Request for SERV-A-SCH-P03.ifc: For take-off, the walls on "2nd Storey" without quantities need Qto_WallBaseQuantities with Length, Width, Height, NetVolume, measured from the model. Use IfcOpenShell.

First a look at what the model holds.

```python
import ifcopenshell
import ifcopenshell.util.element
import ifcopenshell.util.unit

model = ifcopenshell.open("SERV-A-SCH-P03.ifc")
print(model.schema)
for unit_type in ("LENGTHUNIT", "AREAUNIT", "VOLUMEUNIT"):
    print(unit_type, ifcopenshell.util.unit.calculate_unit_scale(model, unit_type))
storey = next(s for s in model.by_type("IfcBuildingStorey") if s.Name == "2nd Storey")
walls = [e for e in ifcopenshell.util.element.get_decomposition(storey) if e.is_a("IfcWall")]
for e in sorted(walls, key=lambda e: e.id()):
    print(e.id(), e.is_a(), e.Name, list(ifcopenshell.util.element.get_psets(e, qtos_only=True)), sep=" | ")
```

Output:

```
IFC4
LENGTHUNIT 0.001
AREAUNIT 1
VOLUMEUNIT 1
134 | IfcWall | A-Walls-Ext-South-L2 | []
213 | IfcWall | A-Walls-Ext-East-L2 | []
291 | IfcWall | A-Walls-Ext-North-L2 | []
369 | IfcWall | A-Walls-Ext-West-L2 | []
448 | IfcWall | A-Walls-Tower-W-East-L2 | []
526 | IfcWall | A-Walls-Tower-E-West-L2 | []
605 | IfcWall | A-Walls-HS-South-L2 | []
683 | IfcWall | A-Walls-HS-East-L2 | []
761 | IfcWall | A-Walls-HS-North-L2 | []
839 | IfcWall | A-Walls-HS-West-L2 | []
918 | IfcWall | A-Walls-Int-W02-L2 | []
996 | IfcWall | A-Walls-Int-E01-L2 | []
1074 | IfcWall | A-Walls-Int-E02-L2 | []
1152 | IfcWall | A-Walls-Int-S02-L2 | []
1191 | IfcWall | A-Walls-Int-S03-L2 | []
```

```python
import ifcopenshell
import ifcopenshell.api.pset
import ifcopenshell.geom
import ifcopenshell.util.element
import ifcopenshell.util.shape
import ifcopenshell.util.unit

model = ifcopenshell.open("SERV-A-SCH-P03.ifc")
unit_scale = ifcopenshell.util.unit.calculate_unit_scale(model)
volume_scale = ifcopenshell.util.unit.calculate_unit_scale(model, "VOLUMEUNIT")
settings = ifcopenshell.geom.settings()

storey = next(s for s in model.by_type("IfcBuildingStorey") if s.Name == "2nd Storey")
walls = [e for e in ifcopenshell.util.element.get_decomposition(storey) if e.is_a("IfcWall")]

for e in sorted(walls, key=lambda e: e.id()):
    if ifcopenshell.util.element.get_psets(e, qtos_only=True, should_inherit=False):
        continue
    # Geometry comes back in metres, in the element's own axes.
    shape = ifcopenshell.geom.create_shape(settings, e)
    values = {
        "Length": ifcopenshell.util.shape.get_x(shape.geometry) / unit_scale,
        "Width": ifcopenshell.util.shape.get_y(shape.geometry) / unit_scale,
        "Height": ifcopenshell.util.shape.get_z(shape.geometry) / unit_scale,
        "NetVolume": ifcopenshell.util.shape.get_volume(shape.geometry) / volume_scale,
    }
    qto = ifcopenshell.api.pset.add_qto(model, product=e, name="Qto_WallBaseQuantities")
    ifcopenshell.api.pset.edit_qto(model, qto=qto, properties=values)
    print(e.id(), {k: round(v, 3) for k, v in values.items()})

model.write("SERV-A-SCH-P03_edited.ifc")
```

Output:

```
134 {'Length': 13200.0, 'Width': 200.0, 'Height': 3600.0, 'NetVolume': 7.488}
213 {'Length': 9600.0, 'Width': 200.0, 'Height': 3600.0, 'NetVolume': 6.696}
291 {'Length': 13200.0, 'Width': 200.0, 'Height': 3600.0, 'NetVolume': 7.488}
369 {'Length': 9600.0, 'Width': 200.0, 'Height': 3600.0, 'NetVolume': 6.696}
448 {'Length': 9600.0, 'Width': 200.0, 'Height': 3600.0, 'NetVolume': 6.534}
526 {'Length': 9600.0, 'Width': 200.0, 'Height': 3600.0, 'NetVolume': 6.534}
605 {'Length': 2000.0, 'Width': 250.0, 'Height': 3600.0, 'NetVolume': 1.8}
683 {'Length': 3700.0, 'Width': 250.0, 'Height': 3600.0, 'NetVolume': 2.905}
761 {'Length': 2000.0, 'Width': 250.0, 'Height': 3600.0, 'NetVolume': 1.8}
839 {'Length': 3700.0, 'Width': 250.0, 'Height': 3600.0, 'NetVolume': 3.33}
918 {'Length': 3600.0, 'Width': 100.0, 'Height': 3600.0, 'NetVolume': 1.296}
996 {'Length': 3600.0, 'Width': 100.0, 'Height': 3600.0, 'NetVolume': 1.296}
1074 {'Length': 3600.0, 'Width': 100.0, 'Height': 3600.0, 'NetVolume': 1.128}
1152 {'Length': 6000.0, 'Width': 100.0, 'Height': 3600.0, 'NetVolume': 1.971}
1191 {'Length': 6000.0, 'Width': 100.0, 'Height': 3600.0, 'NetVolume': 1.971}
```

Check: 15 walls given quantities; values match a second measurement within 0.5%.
